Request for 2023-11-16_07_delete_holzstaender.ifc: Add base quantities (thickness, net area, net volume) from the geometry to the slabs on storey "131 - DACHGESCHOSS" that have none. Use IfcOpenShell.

First a look at what the model holds.

```python
import ifcopenshell
import ifcopenshell.util.element
import ifcopenshell.util.unit

model = ifcopenshell.open("2023-11-16_07_delete_holzstaender.ifc")
print(model.schema)
for unit_type in ("LENGTHUNIT", "AREAUNIT", "VOLUMEUNIT"):
    print(unit_type, ifcopenshell.util.unit.calculate_unit_scale(model, unit_type))
storey = next(s for s in model.by_type("IfcBuildingStorey") if s.Name == "131 - DACHGESCHOSS")
slabs = [e for e in ifcopenshell.util.element.get_decomposition(storey) if e.is_a("IfcSlab")]
for e in sorted(slabs, key=lambda e: e.id()):
    print(e.id(), e.is_a(), e.Name, list(ifcopenshell.util.element.get_psets(e, qtos_only=True)), sep=" | ")
```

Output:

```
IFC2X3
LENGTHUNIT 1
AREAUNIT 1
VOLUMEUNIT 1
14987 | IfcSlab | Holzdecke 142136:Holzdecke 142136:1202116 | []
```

```python
import ifcopenshell
import ifcopenshell.api.pset
import ifcopenshell.geom
import ifcopenshell.util.element
import ifcopenshell.util.shape
import ifcopenshell.util.unit

model = ifcopenshell.open("2023-11-16_07_delete_holzstaender.ifc")
unit_scale = ifcopenshell.util.unit.calculate_unit_scale(model)
area_scale = ifcopenshell.util.unit.calculate_unit_scale(model, "AREAUNIT")
volume_scale = ifcopenshell.util.unit.calculate_unit_scale(model, "VOLUMEUNIT")
settings = ifcopenshell.geom.settings()

storey = next(s for s in model.by_type("IfcBuildingStorey") if s.Name == "131 - DACHGESCHOSS")
slabs = [e for e in ifcopenshell.util.element.get_decomposition(storey) if e.is_a("IfcSlab")]

for e in sorted(slabs, key=lambda e: e.id()):
    if ifcopenshell.util.element.get_psets(e, qtos_only=True, should_inherit=False):
        continue
    # Geometry comes back in metres, in the element's own axes.
    shape = ifcopenshell.geom.create_shape(settings, e)
    values = {
        "Width": ifcopenshell.util.shape.get_z(shape.geometry) / unit_scale,
        "NetArea": ifcopenshell.util.shape.get_footprint_area(shape.geometry) / area_scale,
        "NetVolume": ifcopenshell.util.shape.get_volume(shape.geometry) / volume_scale,
    }
    qto = ifcopenshell.api.pset.add_qto(model, product=e, name="BaseQuantities")
    ifcopenshell.api.pset.edit_qto(model, qto=qto, properties=values)
    print(e.id(), {k: round(v, 3) for k, v in values.items()})

model.write("2023-11-16_07_delete_holzstaender_v2.ifc")
```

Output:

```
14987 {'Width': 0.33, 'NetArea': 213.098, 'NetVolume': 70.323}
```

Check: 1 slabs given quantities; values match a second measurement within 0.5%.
